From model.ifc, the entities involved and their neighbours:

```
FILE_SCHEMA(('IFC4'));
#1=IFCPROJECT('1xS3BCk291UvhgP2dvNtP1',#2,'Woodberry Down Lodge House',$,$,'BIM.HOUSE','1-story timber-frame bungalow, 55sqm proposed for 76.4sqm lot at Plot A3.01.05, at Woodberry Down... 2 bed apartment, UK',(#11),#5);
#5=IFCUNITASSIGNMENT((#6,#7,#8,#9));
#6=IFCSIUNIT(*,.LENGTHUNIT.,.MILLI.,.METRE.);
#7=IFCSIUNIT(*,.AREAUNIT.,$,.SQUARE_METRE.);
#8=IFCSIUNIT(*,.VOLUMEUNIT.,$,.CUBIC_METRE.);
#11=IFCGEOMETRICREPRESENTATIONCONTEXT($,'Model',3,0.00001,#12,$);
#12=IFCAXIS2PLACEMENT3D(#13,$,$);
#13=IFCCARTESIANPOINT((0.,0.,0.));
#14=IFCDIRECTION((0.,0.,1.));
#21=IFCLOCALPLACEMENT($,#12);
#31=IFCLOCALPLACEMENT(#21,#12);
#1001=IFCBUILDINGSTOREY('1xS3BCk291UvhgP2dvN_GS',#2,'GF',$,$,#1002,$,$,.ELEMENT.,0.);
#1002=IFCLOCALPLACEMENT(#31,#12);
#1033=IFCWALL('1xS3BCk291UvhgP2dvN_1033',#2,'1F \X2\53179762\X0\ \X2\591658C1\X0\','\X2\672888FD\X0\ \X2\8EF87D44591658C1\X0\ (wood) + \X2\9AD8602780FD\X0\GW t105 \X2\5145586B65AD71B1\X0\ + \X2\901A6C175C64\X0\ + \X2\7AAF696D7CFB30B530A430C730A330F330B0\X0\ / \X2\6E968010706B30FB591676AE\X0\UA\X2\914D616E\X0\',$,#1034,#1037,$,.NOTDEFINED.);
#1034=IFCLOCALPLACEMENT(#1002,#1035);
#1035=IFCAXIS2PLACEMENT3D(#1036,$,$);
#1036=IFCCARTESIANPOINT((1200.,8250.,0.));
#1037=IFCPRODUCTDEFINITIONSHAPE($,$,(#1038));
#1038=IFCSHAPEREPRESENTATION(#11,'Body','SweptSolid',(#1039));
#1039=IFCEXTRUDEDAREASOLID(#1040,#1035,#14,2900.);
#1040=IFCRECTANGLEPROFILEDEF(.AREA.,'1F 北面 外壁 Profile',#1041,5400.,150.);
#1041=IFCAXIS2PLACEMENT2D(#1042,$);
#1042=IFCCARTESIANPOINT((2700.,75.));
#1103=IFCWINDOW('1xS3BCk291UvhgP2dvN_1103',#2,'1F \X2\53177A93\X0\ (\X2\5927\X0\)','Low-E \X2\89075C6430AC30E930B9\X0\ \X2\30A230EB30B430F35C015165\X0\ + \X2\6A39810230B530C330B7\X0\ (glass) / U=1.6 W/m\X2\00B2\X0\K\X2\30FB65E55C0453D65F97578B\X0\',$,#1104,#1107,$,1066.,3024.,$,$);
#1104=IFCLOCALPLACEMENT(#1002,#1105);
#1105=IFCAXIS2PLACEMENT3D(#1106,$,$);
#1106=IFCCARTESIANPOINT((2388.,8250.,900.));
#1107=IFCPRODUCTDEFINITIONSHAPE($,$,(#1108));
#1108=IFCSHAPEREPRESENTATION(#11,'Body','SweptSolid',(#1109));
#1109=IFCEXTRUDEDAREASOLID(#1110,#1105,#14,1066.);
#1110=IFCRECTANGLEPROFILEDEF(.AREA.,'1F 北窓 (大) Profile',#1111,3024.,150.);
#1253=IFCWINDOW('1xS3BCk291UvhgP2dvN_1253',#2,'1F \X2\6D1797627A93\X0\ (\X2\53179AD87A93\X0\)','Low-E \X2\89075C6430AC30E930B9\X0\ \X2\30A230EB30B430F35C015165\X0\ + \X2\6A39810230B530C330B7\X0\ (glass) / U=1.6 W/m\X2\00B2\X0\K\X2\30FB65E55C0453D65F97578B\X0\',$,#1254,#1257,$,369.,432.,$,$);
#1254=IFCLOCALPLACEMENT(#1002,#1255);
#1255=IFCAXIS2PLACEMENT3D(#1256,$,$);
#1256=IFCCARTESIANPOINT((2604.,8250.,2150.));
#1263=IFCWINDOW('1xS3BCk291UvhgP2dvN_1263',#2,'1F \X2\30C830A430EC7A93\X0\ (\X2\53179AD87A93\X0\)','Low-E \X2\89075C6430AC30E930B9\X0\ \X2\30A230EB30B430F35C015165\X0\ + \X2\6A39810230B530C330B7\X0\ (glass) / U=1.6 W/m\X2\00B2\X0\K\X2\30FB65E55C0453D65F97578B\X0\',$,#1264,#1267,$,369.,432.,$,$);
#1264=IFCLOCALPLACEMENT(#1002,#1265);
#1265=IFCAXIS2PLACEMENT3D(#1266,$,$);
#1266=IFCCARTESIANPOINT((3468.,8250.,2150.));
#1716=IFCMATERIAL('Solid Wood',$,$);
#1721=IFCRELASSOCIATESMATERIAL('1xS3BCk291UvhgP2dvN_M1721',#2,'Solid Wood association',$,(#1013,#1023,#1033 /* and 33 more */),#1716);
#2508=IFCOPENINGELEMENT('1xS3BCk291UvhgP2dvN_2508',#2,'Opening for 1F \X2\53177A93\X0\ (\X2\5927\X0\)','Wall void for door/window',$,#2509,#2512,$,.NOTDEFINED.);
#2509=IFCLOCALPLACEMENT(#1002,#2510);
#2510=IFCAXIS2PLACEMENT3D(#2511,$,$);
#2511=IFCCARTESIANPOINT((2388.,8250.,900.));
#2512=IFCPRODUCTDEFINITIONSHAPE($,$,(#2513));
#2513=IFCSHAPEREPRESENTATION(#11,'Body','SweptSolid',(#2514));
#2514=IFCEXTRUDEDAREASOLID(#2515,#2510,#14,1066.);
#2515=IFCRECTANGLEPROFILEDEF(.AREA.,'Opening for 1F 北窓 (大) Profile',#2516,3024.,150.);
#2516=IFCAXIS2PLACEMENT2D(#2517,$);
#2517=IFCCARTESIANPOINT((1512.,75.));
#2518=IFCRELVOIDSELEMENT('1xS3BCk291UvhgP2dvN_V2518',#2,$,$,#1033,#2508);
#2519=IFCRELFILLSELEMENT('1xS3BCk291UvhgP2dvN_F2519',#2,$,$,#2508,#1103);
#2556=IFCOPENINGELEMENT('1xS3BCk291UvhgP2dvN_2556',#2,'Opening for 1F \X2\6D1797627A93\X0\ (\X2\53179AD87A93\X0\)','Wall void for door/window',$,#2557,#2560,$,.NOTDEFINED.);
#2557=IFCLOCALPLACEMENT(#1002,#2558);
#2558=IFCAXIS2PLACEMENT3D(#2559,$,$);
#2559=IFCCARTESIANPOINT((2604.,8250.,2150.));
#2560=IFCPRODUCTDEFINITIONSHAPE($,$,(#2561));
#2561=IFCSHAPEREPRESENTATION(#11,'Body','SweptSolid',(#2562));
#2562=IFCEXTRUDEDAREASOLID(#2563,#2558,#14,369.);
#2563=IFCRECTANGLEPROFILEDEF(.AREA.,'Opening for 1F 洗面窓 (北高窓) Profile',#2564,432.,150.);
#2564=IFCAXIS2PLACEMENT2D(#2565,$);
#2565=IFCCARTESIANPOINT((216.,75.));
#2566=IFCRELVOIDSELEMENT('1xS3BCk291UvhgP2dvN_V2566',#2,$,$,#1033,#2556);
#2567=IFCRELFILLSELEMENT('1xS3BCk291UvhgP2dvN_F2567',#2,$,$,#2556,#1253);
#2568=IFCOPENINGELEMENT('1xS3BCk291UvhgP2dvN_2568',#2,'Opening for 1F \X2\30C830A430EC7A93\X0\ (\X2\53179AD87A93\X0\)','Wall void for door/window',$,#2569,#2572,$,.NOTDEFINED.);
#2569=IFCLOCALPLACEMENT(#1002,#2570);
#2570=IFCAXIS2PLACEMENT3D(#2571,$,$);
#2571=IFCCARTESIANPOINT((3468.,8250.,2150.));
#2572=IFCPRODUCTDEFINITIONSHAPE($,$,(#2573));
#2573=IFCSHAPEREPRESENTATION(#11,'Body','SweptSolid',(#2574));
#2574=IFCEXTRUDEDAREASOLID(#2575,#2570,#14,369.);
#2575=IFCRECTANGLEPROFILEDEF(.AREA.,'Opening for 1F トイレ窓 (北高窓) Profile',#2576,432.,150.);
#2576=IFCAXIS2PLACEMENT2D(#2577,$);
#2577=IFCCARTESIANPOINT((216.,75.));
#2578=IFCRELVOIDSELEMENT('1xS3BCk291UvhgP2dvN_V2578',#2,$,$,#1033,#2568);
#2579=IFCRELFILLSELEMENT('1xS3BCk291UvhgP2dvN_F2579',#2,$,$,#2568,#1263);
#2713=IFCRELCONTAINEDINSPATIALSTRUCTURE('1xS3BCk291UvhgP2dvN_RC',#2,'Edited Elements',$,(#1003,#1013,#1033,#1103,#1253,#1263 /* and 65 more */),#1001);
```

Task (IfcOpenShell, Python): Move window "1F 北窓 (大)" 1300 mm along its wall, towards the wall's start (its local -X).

```python
import ifcopenshell
import ifcopenshell.api.geometry
import ifcopenshell.util.placement
import ifcopenshell.util.unit

model = ifcopenshell.open("model.ifc")
unit_scale = ifcopenshell.util.unit.calculate_unit_scale(model)

window = model.by_guid("1xS3BCk291UvhgP2dvN_1103")
opening = window.FillsVoids[0].RelatingOpeningElement
wall = opening.VoidsElements[0].RelatingBuildingElement

wall_matrix = ifcopenshell.util.placement.get_local_placement(wall.ObjectPlacement)
shift = wall_matrix[:3, 0] * -1.3 / unit_scale
before = ifcopenshell.util.placement.get_local_placement(window.ObjectPlacement)[:3, 3].copy()

# The window is not placed relative to its opening, so move both.
for product in (opening, window):
    matrix = ifcopenshell.util.placement.get_local_placement(product.ObjectPlacement)
    matrix[:3, 3] += shift
    ifcopenshell.api.geometry.edit_object_placement(model, product=product, matrix=matrix, is_si=False)

after = ifcopenshell.util.placement.get_local_placement(window.ObjectPlacement)[:3, 3]
print("window moved by", (after - before).round(3) + 0.0)

model.write("model_rev.ifc")
```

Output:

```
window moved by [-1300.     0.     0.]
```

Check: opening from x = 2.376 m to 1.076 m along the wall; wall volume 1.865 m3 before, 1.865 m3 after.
